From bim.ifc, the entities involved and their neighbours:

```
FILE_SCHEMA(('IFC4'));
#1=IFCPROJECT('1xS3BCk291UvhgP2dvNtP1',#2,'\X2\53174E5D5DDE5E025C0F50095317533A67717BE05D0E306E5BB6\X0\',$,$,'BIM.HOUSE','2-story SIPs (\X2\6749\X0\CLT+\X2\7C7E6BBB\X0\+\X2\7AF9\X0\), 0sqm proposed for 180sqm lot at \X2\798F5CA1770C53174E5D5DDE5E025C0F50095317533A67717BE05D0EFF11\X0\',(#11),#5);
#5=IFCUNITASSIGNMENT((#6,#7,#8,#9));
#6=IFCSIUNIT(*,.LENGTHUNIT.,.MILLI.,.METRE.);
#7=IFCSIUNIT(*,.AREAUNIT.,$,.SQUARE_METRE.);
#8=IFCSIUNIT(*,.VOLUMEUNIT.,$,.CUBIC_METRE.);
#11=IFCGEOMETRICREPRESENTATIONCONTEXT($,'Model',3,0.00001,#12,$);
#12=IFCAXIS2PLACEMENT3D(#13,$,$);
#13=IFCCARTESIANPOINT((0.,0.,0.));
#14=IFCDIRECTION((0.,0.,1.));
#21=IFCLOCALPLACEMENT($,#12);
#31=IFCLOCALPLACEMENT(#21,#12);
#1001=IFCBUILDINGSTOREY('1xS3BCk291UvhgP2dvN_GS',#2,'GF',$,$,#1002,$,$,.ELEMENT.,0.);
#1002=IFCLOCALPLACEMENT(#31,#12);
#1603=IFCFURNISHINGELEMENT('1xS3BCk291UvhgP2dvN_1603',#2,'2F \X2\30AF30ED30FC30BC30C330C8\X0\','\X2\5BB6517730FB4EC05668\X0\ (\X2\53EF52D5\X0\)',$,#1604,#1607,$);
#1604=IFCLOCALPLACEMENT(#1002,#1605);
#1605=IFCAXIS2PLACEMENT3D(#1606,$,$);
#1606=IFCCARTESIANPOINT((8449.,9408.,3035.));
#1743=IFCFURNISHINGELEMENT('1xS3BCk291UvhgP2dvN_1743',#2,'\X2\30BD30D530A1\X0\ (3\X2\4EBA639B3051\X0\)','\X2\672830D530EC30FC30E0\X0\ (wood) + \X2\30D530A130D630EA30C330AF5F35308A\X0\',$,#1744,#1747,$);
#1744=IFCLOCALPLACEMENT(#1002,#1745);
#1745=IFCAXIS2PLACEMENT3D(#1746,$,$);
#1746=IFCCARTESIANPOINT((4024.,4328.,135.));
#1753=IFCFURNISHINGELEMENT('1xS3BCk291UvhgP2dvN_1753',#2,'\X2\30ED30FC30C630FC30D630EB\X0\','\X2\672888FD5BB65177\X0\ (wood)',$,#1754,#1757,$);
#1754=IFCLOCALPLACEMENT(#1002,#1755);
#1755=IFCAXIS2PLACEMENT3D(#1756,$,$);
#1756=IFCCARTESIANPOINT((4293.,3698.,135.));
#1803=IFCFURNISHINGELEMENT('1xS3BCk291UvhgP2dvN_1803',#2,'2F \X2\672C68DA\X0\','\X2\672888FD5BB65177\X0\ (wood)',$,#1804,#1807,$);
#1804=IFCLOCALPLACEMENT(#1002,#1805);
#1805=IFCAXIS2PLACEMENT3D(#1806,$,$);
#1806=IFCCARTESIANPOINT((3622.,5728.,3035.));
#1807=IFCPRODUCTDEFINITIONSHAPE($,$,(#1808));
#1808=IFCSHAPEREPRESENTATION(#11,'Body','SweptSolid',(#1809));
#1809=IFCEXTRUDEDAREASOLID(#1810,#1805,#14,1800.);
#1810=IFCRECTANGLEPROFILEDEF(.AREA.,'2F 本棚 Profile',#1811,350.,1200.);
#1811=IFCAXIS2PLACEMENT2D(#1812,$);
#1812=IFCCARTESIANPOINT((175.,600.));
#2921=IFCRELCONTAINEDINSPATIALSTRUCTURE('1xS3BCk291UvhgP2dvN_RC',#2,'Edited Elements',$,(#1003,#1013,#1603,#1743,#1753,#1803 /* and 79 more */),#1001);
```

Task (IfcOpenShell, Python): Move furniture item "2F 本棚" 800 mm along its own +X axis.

```python
import ifcopenshell
import ifcopenshell.api.geometry
import ifcopenshell.util.placement

model = ifcopenshell.open("bim.ifc")

item = model.by_guid("1xS3BCk291UvhgP2dvN_1803")
matrix = ifcopenshell.util.placement.get_local_placement(item.ObjectPlacement)
matrix[:3, 3] += matrix[:3, 0] * 800.0
ifcopenshell.api.geometry.edit_object_placement(model, product=item, matrix=matrix, is_si=False)

print(ifcopenshell.util.placement.get_local_placement(item.ObjectPlacement).round(3) + 0.0)

model.write("bim-out.ifc")
```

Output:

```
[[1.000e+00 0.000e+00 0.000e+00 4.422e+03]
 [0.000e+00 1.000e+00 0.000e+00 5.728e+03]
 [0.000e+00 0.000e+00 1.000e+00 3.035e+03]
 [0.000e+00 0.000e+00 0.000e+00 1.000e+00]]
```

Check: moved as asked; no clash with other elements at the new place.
